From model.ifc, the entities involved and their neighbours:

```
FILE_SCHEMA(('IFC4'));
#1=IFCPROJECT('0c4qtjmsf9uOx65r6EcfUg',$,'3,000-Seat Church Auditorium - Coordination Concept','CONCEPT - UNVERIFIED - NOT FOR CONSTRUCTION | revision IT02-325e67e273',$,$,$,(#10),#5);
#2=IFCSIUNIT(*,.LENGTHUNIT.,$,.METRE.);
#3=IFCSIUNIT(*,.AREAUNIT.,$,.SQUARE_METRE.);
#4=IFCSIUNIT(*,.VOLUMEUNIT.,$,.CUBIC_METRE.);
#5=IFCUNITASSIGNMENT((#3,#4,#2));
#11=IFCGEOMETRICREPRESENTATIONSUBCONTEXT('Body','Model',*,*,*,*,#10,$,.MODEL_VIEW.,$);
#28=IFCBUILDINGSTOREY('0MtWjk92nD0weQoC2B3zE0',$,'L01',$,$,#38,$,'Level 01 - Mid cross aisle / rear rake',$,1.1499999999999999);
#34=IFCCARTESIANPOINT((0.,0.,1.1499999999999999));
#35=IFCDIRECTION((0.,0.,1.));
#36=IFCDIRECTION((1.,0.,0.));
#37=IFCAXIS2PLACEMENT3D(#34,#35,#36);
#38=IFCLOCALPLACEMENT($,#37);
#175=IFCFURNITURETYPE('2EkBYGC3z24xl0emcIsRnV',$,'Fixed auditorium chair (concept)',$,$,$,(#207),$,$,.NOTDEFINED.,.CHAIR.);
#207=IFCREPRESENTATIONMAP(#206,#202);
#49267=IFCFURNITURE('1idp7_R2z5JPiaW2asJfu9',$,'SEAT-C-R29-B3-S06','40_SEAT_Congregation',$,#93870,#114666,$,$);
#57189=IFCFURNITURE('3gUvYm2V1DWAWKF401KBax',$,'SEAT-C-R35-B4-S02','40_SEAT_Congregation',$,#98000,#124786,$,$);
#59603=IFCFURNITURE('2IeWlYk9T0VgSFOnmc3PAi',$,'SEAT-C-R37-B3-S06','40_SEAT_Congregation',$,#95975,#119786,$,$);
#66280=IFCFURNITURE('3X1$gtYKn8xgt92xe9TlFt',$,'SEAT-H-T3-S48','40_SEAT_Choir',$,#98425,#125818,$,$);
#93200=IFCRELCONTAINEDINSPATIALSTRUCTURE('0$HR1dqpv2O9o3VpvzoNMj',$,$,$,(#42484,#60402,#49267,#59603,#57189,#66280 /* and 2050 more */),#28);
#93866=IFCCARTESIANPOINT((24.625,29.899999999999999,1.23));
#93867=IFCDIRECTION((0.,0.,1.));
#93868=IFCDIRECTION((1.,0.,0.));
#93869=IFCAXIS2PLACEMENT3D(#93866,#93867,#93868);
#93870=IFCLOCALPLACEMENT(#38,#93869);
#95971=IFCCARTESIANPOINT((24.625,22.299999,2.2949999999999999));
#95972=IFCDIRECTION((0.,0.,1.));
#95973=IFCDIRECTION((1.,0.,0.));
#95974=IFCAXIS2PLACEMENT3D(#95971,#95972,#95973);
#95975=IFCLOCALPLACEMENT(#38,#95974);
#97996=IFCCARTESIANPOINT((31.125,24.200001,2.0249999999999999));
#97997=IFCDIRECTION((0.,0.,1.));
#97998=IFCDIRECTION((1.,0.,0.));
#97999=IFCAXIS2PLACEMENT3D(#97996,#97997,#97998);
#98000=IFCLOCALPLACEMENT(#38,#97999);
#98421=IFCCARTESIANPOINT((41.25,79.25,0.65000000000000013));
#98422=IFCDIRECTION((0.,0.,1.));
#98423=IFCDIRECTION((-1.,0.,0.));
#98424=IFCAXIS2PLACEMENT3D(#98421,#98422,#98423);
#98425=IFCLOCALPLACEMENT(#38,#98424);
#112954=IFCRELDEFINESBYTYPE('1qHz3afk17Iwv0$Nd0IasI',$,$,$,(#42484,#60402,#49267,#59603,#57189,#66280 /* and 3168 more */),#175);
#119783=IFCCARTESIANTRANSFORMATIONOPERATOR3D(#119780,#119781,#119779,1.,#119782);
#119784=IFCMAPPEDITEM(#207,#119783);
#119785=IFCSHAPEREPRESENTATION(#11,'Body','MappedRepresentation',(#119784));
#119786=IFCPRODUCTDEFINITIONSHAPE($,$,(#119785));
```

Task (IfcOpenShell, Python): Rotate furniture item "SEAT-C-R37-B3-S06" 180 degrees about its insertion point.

```python
import ifcopenshell
import ifcopenshell.api.geometry
import ifcopenshell.util.placement

model = ifcopenshell.open("model.ifc")

item = model.by_guid("2IeWlYk9T0VgSFOnmc3PAi")
matrix = ifcopenshell.util.placement.get_local_placement(item.ObjectPlacement)
matrix = matrix @ ifcopenshell.util.placement.rotation(180, "Z")
ifcopenshell.api.geometry.edit_object_placement(model, product=item, matrix=matrix, is_si=False)

print(ifcopenshell.util.placement.get_local_placement(item.ObjectPlacement).round(3) + 0.0)

model.write("model_rev.ifc")
```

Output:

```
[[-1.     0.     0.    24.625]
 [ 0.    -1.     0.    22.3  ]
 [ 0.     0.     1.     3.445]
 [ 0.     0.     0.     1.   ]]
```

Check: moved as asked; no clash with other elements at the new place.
